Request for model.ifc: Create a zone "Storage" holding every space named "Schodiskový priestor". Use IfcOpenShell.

First a look at what the model holds.

```python
import ifcopenshell

model = ifcopenshell.open("model.ifc")
print(model.schema)
seen = {}
for space in model.by_type("IfcSpace"):
    seen[space.LongName] = seen.get(space.LongName, 0) + 1
for name, count in sorted(seen.items(), key=str):
    print(count, "x", name)
print("zones:", [z.Name for z in model.by_type("IfcZone")][:20])
```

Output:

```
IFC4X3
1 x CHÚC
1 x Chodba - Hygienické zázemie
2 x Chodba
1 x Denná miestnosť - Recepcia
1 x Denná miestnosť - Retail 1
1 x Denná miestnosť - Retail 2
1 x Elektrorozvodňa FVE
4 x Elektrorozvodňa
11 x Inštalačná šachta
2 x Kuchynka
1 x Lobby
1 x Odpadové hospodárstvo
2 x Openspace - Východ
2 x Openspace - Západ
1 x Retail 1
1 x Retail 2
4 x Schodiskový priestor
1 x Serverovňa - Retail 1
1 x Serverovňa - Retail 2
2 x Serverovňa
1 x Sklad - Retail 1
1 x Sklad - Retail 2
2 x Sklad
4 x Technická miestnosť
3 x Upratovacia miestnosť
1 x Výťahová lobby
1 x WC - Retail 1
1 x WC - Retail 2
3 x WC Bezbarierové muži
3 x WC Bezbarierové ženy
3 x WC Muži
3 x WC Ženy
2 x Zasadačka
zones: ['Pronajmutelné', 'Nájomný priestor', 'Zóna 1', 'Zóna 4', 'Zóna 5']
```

```python
import ifcopenshell
import ifcopenshell.api.group
import ifcopenshell.api.root

model = ifcopenshell.open("model.ifc")

names = {"Schodiskový priestor"}
spaces = [s for s in model.by_type("IfcSpace") if s.LongName in names]

zone = ifcopenshell.api.root.create_entity(model, ifc_class="IfcZone", name="Storage")
ifcopenshell.api.group.assign_group(model, products=spaces, group=zone)
print(len(spaces), "spaces in", zone.Name)

model.write("model_updated.ifc")
```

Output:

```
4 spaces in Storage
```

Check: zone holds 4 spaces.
